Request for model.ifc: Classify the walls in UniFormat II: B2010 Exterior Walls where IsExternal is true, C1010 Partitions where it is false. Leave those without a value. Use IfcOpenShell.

First a look at what the model holds.

```python
import ifcopenshell
import ifcopenshell.util.element

model = ifcopenshell.open("model.ifc")
print(model.schema)
print("classifications:", [c.Name for c in model.by_type("IfcClassification")])
values = [ifcopenshell.util.element.get_pset(e, "Pset_WallCommon", "IsExternal") for e in model.by_type("IfcWall")]
for value in (True, False, None):
    print("IsExternal", value, values.count(value))
```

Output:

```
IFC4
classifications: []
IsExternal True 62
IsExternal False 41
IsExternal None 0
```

```python
import ifcopenshell
import ifcopenshell.api.classification
import ifcopenshell.util.element

model = ifcopenshell.open("model.ifc")

system = ifcopenshell.api.classification.add_classification(model, classification="UniFormat II")

walls = model.by_type("IfcWall")
external = {e: ifcopenshell.util.element.get_pset(e, "Pset_WallCommon", "IsExternal") for e in walls}
for flag, code, name in ((True, "B2010", "Exterior Walls"), (False, "C1010", "Partitions")):
    products = [e for e in walls if external[e] is flag]
    ifcopenshell.api.classification.add_reference(
        model, products=products, classification=system, identification=code, name=name
    )
    print(code, len(products))

model.write("model_updated.ifc")
```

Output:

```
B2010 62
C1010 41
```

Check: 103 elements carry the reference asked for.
